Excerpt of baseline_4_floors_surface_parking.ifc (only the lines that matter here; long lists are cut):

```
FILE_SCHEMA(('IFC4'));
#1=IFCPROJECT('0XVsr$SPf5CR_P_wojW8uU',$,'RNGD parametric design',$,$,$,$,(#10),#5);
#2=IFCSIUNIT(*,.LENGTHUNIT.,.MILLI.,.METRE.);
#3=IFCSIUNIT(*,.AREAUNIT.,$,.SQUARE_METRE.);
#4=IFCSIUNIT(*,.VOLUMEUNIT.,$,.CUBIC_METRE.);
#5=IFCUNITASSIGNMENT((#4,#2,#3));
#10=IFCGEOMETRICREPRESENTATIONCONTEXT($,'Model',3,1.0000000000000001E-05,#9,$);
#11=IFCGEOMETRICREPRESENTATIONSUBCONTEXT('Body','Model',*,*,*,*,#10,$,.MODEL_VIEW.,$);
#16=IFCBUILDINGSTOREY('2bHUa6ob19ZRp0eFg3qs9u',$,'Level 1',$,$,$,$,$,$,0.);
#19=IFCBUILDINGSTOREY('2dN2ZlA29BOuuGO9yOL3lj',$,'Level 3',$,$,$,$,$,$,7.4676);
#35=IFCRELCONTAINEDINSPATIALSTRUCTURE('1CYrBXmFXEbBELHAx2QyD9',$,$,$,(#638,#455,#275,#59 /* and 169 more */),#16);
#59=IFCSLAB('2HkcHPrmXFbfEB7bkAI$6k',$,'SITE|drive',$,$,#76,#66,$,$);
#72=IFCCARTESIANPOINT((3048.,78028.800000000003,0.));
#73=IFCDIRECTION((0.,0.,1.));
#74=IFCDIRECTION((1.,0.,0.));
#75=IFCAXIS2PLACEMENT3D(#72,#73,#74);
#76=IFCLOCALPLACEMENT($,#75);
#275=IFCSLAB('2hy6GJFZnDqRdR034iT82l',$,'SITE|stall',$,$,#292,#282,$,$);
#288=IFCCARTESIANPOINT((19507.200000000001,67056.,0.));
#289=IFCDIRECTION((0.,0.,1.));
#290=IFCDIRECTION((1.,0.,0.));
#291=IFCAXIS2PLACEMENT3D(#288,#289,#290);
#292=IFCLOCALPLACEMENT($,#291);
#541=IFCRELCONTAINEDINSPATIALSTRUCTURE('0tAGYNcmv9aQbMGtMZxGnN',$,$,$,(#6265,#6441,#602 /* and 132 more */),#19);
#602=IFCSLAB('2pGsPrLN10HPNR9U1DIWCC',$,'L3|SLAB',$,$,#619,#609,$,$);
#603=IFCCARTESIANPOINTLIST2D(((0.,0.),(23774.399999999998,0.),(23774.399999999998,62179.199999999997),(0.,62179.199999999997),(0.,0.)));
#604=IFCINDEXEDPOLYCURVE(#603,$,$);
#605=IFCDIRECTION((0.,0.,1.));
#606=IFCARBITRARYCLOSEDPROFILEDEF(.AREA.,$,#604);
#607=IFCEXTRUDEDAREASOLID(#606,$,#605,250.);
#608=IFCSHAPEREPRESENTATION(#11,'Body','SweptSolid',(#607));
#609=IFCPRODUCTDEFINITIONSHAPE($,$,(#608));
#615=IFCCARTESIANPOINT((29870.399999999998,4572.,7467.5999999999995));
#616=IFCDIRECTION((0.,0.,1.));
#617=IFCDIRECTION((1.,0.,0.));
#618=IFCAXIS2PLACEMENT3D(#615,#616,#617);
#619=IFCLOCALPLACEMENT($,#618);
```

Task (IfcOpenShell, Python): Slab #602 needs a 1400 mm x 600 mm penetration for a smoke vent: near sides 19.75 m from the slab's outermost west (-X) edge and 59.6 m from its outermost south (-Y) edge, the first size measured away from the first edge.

```python
import numpy as np
import ifcopenshell
import ifcopenshell.api.feature
import ifcopenshell.api.geometry
import ifcopenshell.api.root
import ifcopenshell.geom
import ifcopenshell.util.placement
import ifcopenshell.util.representation
import ifcopenshell.util.shape
import ifcopenshell.util.unit

model = ifcopenshell.open("baseline_4_floors_surface_parking.ifc")
unit_scale = ifcopenshell.util.unit.calculate_unit_scale(model)
settings = ifcopenshell.geom.settings()


def volume(element):
    """Net volume in cubic metres, openings subtracted."""
    shape = ifcopenshell.geom.create_shape(settings, element)
    return ifcopenshell.util.shape.get_volume(shape.geometry)


slab = model.by_id(602)
before = volume(slab)

# Extent in the slab's own axes, in metres. The edges named are its -X and -Y sides.
slab_shape = ifcopenshell.geom.create_shape(settings, slab)
vertices = ifcopenshell.util.shape.get_vertices(slab_shape.geometry)
x_min, y_min, bottom = vertices.min(axis=0)
top = vertices[:, 2].max()

opening = ifcopenshell.api.root.create_entity(model, ifc_class="IfcOpeningElement", name="Smoke vent opening", predefined_type="OPENING")
context = ifcopenshell.util.representation.get_context(model, "Model", "Body", "MODEL_VIEW")
width, depth = 1.4, 0.6
outline = [(0.0, 0.0), (width, 0.0), (width, depth), (0.0, depth), (0.0, 0.0)]
# Overshoot both faces by 50 mm so the cut is clean.
shape = ifcopenshell.api.geometry.add_slab_representation(
    model, context=context, depth=top - bottom + 0.1, polyline=outline
)
ifcopenshell.api.geometry.assign_representation(model, product=opening, representation=shape)

matrix = ifcopenshell.util.placement.get_local_placement(slab.ObjectPlacement)
matrix[:, 3] = matrix @ np.append(np.array([x_min + 19.75, y_min + 59.6, bottom - 0.05]) / unit_scale, 1.0)
ifcopenshell.api.geometry.edit_object_placement(model, product=opening, matrix=matrix, is_si=False)
ifcopenshell.api.feature.add_feature(model, feature=opening, element=slab)

after = volume(slab)

print(f"slab volume {before:.3f} -> {after:.3f} m3")

model.write("baseline_4_floors_surface_parking_updated.ifc")
```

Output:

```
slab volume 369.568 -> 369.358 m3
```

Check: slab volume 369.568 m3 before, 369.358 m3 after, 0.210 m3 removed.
